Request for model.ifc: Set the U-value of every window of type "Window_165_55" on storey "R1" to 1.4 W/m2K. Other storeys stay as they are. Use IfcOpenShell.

First a look at what the model holds.

```python
import ifcopenshell
import ifcopenshell.util.element

model = ifcopenshell.open("model.ifc")
print(model.schema)
storey = next(s for s in model.by_type("IfcBuildingStorey") if s.Name == "R1")
windows = [e for e in ifcopenshell.util.element.get_decomposition(storey) if e.is_a("IfcWindow")]
seen = {}
for e in windows:
    element_type = ifcopenshell.util.element.get_type(e)
    key = (element_type.Name if element_type != e and element_type else None, ifcopenshell.util.element.get_pset(e, "Pset_WindowCommon", "ThermalTransmittance"))
    seen[key] = seen.get(key, 0) + 1
for (name, value), count in sorted(seen.items(), key=str):
    print(count, "x", name, "|", value)
```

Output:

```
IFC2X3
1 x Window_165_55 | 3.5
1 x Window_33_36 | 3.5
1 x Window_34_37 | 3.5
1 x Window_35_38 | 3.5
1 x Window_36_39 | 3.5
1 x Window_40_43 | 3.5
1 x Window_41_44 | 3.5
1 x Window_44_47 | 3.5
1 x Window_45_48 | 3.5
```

```python
import ifcopenshell
import ifcopenshell.api.pset
import ifcopenshell.util.element

model = ifcopenshell.open("model.ifc")

storey = next(s for s in model.by_type("IfcBuildingStorey") if s.Name == "R1")
windows = [e for e in ifcopenshell.util.element.get_decomposition(storey) if e.is_a("IfcWindow")]

count = 0
for e in windows:
    element_type = ifcopenshell.util.element.get_type(e)
    if element_type in (None, e) or element_type.Name != "Window_165_55":
        continue
    # add_pset returns the element's existing set when there is one.
    pset = ifcopenshell.api.pset.add_pset(model, product=e, name="Pset_WindowCommon")
    ifcopenshell.api.pset.edit_pset(model, pset=pset, properties={"ThermalTransmittance": 1.4})
    count += 1

print(count, "windows updated")

model.write("model_v2.ifc")
```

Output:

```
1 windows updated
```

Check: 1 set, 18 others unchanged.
